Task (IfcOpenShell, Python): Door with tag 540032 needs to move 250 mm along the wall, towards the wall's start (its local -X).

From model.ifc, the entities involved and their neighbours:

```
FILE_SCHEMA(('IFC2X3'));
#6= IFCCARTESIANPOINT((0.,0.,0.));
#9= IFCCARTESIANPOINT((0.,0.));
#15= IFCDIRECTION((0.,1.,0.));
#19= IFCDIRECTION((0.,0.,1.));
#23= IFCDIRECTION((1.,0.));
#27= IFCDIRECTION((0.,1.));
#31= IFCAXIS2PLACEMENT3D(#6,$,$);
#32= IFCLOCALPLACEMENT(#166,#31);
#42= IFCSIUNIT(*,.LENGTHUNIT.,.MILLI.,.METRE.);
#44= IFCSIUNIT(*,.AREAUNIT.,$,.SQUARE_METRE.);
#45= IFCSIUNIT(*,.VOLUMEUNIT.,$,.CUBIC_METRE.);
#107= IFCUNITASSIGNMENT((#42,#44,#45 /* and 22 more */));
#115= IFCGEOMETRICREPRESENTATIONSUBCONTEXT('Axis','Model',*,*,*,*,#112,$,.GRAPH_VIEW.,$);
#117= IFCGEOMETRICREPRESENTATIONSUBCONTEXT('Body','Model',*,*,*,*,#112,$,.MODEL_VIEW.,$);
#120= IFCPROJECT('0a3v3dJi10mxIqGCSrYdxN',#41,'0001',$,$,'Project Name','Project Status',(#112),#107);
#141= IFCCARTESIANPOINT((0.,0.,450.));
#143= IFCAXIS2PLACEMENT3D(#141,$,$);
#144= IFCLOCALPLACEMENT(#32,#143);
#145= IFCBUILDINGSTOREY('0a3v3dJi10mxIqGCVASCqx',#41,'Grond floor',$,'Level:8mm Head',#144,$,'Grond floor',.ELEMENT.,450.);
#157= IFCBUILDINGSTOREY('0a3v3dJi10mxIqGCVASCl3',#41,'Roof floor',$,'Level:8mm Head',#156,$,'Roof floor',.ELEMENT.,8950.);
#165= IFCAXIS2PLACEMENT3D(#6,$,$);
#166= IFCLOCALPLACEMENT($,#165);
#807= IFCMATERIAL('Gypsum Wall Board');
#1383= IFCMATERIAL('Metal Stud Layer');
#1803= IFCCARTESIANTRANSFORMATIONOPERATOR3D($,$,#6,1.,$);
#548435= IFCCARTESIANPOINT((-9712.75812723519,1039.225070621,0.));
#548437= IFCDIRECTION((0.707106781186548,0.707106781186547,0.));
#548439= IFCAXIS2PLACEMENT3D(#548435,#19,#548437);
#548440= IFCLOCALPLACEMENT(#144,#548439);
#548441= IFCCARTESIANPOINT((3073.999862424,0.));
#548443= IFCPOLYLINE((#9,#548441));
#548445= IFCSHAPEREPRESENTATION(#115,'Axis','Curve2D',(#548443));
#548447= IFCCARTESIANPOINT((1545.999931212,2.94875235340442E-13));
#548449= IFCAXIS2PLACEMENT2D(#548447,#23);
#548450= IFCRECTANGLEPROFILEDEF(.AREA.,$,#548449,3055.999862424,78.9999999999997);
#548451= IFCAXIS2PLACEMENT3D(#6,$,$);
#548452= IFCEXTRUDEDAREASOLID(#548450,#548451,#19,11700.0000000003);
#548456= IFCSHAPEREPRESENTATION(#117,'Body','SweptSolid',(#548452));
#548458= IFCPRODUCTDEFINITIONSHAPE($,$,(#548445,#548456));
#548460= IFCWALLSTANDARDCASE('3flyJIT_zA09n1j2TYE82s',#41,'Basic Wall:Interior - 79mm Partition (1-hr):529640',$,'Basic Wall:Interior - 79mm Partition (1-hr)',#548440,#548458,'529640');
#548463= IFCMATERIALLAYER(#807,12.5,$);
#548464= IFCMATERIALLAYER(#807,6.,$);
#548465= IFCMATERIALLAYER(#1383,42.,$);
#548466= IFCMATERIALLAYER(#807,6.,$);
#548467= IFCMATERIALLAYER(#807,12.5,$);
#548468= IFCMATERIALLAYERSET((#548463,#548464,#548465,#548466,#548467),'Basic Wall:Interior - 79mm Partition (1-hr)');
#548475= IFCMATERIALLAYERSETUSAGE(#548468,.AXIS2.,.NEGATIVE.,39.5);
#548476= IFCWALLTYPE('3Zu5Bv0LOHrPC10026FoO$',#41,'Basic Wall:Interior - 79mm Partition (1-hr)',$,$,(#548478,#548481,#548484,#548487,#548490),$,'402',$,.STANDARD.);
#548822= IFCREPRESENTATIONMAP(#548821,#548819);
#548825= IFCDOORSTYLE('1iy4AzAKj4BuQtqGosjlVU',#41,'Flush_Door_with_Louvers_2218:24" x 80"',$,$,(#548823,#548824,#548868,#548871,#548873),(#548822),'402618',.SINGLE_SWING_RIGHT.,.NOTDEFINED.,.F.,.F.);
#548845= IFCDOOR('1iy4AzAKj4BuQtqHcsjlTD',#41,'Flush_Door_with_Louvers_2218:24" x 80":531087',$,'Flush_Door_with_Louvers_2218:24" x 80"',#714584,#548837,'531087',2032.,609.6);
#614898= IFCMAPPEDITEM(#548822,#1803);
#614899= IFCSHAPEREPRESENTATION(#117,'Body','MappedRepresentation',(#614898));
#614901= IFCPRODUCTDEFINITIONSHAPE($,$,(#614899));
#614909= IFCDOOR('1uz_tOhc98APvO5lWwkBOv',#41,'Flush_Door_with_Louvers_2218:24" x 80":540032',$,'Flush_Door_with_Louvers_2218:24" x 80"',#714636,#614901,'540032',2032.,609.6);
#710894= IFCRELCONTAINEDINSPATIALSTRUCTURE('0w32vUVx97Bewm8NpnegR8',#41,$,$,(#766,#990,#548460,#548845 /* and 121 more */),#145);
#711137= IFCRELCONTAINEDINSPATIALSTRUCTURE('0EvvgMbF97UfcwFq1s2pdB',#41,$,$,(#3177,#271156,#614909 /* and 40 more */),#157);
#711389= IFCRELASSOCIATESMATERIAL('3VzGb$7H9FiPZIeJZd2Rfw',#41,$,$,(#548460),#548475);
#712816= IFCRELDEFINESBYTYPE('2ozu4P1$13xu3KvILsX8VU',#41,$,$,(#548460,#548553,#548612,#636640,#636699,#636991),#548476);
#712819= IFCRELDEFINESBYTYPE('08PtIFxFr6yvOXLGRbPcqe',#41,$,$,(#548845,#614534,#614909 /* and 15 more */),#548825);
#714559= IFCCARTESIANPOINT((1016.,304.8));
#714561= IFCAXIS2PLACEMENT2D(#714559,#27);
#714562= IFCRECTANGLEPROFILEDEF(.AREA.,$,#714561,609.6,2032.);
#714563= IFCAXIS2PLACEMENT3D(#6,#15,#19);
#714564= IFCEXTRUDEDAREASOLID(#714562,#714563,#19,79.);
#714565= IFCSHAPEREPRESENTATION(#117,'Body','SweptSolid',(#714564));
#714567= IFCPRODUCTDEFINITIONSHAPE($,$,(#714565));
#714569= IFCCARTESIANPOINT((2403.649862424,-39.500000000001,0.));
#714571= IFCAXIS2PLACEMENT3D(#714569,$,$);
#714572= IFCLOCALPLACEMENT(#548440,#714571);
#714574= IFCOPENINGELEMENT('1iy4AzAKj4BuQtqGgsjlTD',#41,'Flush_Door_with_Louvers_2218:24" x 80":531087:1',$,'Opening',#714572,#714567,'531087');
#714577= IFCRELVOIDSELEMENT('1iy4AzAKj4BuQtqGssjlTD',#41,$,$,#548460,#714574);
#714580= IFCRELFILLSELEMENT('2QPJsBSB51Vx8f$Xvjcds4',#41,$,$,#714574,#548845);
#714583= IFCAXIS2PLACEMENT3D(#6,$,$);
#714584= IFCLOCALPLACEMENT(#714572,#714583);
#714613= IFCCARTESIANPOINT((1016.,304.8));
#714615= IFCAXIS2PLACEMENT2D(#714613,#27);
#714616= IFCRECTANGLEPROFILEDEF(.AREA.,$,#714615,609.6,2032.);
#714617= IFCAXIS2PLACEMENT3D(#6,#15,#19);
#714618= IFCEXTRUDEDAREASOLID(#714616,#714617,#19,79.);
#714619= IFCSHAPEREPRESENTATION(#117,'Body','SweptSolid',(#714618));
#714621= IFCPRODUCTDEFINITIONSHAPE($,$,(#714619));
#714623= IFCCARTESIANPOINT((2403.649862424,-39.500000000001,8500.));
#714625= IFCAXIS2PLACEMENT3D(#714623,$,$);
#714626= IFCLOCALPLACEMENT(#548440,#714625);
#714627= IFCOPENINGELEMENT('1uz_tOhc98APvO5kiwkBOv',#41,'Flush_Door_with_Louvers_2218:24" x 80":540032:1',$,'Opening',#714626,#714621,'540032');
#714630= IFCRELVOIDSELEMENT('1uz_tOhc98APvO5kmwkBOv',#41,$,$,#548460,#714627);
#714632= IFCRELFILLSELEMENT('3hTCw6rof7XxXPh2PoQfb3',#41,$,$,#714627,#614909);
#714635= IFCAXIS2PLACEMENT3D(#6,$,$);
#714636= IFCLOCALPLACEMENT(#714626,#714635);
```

```python
import ifcopenshell
import ifcopenshell.api.geometry
import ifcopenshell.util.placement

model = ifcopenshell.open("model.ifc")

door = model.by_guid("1uz_tOhc98APvO5lWwkBOv")
opening = door.FillsVoids[0].RelatingOpeningElement
wall = opening.VoidsElements[0].RelatingBuildingElement

wall_matrix = ifcopenshell.util.placement.get_local_placement(wall.ObjectPlacement)
shift = wall_matrix[:3, 0] * -250.0
before = ifcopenshell.util.placement.get_local_placement(door.ObjectPlacement)[:3, 3].copy()

# The door is placed relative to its opening, so it follows when the opening moves.
matrix = ifcopenshell.util.placement.get_local_placement(opening.ObjectPlacement)
matrix[:3, 3] += shift
ifcopenshell.api.geometry.edit_object_placement(
    model, product=opening, matrix=matrix, is_si=False, should_transform_children=True
)

after = ifcopenshell.util.placement.get_local_placement(door.ObjectPlacement)[:3, 3]
print("door moved by", (after - before).round(3) + 0.0)

model.write("model_updated.ifc")
```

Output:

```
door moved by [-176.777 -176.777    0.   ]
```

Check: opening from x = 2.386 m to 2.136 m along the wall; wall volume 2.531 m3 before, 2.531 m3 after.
